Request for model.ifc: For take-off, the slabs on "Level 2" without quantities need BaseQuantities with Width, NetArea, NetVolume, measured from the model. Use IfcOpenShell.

First a look at what the model holds.

```python
import ifcopenshell
import ifcopenshell.util.element
import ifcopenshell.util.unit

model = ifcopenshell.open("model.ifc")
print(model.schema)
for unit_type in ("LENGTHUNIT", "AREAUNIT", "VOLUMEUNIT"):
    print(unit_type, ifcopenshell.util.unit.calculate_unit_scale(model, unit_type))
storey = next(s for s in model.by_type("IfcBuildingStorey") if s.Name == "Level 2")
slabs = [e for e in ifcopenshell.util.element.get_decomposition(storey) if e.is_a("IfcSlab")]
for e in sorted(slabs, key=lambda e: e.id()):
    print(e.id(), e.is_a(), e.Name, list(ifcopenshell.util.element.get_psets(e, qtos_only=True)), sep=" | ")
```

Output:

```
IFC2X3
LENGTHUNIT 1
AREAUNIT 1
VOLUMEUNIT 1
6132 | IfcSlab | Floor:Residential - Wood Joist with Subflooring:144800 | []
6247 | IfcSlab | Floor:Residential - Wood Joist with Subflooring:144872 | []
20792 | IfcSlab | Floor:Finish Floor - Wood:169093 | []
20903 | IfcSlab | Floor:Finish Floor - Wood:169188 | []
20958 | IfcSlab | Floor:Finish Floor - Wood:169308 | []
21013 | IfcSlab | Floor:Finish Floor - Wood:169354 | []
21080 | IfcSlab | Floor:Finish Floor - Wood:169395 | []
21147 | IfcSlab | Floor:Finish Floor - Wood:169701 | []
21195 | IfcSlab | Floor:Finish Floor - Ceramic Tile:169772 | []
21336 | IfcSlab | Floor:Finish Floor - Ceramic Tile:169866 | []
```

```python
import ifcopenshell
import ifcopenshell.api.pset
import ifcopenshell.geom
import ifcopenshell.util.element
import ifcopenshell.util.shape
import ifcopenshell.util.unit

model = ifcopenshell.open("model.ifc")
unit_scale = ifcopenshell.util.unit.calculate_unit_scale(model)
area_scale = ifcopenshell.util.unit.calculate_unit_scale(model, "AREAUNIT")
volume_scale = ifcopenshell.util.unit.calculate_unit_scale(model, "VOLUMEUNIT")
settings = ifcopenshell.geom.settings()

storey = next(s for s in model.by_type("IfcBuildingStorey") if s.Name == "Level 2")
slabs = [e for e in ifcopenshell.util.element.get_decomposition(storey) if e.is_a("IfcSlab")]

for e in sorted(slabs, key=lambda e: e.id()):
    if ifcopenshell.util.element.get_psets(e, qtos_only=True, should_inherit=False):
        continue
    # Geometry comes back in metres, in the element's own axes.
    shape = ifcopenshell.geom.create_shape(settings, e)
    values = {
        "Width": ifcopenshell.util.shape.get_z(shape.geometry) / unit_scale,
        "NetArea": ifcopenshell.util.shape.get_footprint_area(shape.geometry) / area_scale,
        "NetVolume": ifcopenshell.util.shape.get_volume(shape.geometry) / volume_scale,
    }
    qto = ifcopenshell.api.pset.add_qto(model, product=e, name="BaseQuantities")
    ifcopenshell.api.pset.edit_qto(model, qto=qto, properties=values)
    print(e.id(), {k: round(v, 3) for k, v in values.items()})

model.write("model-out.ifc")
```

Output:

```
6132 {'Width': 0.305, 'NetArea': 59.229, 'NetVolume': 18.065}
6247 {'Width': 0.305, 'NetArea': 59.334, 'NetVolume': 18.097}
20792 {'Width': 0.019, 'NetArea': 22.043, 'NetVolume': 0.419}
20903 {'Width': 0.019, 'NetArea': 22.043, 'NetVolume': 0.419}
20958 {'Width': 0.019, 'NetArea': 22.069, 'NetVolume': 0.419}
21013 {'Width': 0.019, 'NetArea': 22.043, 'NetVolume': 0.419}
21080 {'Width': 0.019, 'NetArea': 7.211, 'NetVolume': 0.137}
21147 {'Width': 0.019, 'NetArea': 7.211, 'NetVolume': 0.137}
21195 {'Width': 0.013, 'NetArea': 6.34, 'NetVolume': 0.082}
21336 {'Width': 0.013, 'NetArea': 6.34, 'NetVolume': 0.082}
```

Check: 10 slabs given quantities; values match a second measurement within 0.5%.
